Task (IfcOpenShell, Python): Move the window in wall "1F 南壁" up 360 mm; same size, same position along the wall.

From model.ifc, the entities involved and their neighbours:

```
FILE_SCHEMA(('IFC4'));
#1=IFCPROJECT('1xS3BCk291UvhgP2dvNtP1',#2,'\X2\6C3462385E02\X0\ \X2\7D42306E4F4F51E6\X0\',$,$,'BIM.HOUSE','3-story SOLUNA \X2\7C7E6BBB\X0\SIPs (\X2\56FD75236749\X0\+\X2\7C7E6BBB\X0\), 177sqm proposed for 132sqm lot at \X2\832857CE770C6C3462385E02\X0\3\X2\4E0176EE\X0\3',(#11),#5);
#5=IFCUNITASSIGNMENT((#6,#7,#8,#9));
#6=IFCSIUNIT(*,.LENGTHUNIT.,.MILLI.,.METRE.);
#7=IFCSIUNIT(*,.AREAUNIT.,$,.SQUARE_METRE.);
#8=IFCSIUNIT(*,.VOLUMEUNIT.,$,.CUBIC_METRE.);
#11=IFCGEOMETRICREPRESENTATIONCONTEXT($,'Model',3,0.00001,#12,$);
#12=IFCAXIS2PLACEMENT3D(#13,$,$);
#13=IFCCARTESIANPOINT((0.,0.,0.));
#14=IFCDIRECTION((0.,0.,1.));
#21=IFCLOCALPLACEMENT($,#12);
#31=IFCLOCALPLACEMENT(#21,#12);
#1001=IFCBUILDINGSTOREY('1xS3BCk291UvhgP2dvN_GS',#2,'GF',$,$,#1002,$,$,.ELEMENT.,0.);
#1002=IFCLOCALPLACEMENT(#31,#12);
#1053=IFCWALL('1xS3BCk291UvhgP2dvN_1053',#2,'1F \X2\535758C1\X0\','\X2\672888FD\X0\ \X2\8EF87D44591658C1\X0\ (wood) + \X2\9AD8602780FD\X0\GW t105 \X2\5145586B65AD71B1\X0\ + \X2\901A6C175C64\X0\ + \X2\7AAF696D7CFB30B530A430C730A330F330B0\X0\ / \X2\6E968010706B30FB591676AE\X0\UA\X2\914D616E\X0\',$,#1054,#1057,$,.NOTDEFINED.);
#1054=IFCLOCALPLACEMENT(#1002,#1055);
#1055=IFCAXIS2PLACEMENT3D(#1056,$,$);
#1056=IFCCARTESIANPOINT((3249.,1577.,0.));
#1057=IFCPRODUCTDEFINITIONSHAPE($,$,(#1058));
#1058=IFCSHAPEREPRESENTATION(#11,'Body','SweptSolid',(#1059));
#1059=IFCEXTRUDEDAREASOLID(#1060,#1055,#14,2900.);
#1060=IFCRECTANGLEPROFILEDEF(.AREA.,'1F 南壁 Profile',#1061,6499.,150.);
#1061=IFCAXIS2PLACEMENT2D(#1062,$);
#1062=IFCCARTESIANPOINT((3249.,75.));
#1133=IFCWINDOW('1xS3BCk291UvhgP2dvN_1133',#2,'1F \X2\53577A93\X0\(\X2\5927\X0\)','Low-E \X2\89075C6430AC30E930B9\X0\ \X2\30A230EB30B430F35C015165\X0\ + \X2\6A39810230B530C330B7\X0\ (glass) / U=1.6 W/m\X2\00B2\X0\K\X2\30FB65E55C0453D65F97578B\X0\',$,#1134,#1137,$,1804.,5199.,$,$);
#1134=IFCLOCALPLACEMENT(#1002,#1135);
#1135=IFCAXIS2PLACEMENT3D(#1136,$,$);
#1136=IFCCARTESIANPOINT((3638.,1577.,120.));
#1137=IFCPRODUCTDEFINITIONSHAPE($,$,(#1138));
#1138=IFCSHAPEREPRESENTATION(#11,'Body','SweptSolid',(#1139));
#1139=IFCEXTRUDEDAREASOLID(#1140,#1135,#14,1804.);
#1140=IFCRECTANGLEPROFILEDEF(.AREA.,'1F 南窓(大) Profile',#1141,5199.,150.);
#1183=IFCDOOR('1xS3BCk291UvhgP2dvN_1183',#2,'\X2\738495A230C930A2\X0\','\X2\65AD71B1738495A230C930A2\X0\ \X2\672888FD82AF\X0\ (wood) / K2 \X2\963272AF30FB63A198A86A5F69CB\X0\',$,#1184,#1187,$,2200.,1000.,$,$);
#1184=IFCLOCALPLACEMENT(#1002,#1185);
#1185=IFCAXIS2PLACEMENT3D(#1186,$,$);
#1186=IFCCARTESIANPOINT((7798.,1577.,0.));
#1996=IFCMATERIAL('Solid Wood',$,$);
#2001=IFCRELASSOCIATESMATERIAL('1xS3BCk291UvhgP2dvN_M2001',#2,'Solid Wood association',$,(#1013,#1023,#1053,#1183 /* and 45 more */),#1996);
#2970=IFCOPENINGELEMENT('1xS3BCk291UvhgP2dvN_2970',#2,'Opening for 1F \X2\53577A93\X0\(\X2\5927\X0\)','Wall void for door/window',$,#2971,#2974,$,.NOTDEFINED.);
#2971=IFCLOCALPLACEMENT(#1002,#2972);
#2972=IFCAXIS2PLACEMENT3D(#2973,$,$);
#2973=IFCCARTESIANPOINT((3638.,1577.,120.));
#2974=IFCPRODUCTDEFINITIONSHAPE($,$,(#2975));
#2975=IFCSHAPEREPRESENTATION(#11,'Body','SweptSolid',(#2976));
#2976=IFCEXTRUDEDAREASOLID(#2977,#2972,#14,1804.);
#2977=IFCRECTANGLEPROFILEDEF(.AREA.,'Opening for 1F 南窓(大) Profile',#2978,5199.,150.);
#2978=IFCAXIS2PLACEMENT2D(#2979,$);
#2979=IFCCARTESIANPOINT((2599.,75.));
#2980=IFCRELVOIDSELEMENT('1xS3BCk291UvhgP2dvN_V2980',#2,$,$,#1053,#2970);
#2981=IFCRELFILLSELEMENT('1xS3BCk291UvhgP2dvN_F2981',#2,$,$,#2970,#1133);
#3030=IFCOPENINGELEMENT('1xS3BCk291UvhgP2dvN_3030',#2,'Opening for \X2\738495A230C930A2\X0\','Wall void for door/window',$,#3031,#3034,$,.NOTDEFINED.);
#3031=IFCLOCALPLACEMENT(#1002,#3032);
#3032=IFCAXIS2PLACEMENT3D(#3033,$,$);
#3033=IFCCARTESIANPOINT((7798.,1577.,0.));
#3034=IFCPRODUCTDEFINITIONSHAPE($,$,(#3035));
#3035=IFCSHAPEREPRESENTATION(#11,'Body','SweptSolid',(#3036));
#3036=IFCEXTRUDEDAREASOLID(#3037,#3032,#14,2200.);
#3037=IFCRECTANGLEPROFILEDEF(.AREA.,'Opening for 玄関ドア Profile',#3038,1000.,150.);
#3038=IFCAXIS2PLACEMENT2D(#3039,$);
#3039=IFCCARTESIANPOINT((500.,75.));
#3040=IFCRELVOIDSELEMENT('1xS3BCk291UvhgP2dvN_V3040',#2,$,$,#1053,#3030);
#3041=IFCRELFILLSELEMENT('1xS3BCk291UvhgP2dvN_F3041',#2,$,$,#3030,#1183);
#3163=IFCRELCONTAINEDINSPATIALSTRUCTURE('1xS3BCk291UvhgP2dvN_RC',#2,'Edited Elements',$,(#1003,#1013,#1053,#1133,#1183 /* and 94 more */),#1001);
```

```python
import numpy as np
import ifcopenshell
import ifcopenshell.api.geometry
import ifcopenshell.util.placement
import ifcopenshell.util.unit

model = ifcopenshell.open("model.ifc")
unit_scale = ifcopenshell.util.unit.calculate_unit_scale(model)

window = model.by_guid("1xS3BCk291UvhgP2dvN_1133")
opening = window.FillsVoids[0].RelatingOpeningElement
dz = 360.0

shift = np.array([0.0, 0.0, dz])
# The window is not placed relative to its opening, so move both.
for product in (opening, window):
    matrix = ifcopenshell.util.placement.get_local_placement(product.ObjectPlacement)
    matrix[:3, 3] += shift
    ifcopenshell.api.geometry.edit_object_placement(model, product=product, matrix=matrix, is_si=False)

print(f"moved by {dz * unit_scale:+.3f} m")

model.write("model_v2.ifc")
```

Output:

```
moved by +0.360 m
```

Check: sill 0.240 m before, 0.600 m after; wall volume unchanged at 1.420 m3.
